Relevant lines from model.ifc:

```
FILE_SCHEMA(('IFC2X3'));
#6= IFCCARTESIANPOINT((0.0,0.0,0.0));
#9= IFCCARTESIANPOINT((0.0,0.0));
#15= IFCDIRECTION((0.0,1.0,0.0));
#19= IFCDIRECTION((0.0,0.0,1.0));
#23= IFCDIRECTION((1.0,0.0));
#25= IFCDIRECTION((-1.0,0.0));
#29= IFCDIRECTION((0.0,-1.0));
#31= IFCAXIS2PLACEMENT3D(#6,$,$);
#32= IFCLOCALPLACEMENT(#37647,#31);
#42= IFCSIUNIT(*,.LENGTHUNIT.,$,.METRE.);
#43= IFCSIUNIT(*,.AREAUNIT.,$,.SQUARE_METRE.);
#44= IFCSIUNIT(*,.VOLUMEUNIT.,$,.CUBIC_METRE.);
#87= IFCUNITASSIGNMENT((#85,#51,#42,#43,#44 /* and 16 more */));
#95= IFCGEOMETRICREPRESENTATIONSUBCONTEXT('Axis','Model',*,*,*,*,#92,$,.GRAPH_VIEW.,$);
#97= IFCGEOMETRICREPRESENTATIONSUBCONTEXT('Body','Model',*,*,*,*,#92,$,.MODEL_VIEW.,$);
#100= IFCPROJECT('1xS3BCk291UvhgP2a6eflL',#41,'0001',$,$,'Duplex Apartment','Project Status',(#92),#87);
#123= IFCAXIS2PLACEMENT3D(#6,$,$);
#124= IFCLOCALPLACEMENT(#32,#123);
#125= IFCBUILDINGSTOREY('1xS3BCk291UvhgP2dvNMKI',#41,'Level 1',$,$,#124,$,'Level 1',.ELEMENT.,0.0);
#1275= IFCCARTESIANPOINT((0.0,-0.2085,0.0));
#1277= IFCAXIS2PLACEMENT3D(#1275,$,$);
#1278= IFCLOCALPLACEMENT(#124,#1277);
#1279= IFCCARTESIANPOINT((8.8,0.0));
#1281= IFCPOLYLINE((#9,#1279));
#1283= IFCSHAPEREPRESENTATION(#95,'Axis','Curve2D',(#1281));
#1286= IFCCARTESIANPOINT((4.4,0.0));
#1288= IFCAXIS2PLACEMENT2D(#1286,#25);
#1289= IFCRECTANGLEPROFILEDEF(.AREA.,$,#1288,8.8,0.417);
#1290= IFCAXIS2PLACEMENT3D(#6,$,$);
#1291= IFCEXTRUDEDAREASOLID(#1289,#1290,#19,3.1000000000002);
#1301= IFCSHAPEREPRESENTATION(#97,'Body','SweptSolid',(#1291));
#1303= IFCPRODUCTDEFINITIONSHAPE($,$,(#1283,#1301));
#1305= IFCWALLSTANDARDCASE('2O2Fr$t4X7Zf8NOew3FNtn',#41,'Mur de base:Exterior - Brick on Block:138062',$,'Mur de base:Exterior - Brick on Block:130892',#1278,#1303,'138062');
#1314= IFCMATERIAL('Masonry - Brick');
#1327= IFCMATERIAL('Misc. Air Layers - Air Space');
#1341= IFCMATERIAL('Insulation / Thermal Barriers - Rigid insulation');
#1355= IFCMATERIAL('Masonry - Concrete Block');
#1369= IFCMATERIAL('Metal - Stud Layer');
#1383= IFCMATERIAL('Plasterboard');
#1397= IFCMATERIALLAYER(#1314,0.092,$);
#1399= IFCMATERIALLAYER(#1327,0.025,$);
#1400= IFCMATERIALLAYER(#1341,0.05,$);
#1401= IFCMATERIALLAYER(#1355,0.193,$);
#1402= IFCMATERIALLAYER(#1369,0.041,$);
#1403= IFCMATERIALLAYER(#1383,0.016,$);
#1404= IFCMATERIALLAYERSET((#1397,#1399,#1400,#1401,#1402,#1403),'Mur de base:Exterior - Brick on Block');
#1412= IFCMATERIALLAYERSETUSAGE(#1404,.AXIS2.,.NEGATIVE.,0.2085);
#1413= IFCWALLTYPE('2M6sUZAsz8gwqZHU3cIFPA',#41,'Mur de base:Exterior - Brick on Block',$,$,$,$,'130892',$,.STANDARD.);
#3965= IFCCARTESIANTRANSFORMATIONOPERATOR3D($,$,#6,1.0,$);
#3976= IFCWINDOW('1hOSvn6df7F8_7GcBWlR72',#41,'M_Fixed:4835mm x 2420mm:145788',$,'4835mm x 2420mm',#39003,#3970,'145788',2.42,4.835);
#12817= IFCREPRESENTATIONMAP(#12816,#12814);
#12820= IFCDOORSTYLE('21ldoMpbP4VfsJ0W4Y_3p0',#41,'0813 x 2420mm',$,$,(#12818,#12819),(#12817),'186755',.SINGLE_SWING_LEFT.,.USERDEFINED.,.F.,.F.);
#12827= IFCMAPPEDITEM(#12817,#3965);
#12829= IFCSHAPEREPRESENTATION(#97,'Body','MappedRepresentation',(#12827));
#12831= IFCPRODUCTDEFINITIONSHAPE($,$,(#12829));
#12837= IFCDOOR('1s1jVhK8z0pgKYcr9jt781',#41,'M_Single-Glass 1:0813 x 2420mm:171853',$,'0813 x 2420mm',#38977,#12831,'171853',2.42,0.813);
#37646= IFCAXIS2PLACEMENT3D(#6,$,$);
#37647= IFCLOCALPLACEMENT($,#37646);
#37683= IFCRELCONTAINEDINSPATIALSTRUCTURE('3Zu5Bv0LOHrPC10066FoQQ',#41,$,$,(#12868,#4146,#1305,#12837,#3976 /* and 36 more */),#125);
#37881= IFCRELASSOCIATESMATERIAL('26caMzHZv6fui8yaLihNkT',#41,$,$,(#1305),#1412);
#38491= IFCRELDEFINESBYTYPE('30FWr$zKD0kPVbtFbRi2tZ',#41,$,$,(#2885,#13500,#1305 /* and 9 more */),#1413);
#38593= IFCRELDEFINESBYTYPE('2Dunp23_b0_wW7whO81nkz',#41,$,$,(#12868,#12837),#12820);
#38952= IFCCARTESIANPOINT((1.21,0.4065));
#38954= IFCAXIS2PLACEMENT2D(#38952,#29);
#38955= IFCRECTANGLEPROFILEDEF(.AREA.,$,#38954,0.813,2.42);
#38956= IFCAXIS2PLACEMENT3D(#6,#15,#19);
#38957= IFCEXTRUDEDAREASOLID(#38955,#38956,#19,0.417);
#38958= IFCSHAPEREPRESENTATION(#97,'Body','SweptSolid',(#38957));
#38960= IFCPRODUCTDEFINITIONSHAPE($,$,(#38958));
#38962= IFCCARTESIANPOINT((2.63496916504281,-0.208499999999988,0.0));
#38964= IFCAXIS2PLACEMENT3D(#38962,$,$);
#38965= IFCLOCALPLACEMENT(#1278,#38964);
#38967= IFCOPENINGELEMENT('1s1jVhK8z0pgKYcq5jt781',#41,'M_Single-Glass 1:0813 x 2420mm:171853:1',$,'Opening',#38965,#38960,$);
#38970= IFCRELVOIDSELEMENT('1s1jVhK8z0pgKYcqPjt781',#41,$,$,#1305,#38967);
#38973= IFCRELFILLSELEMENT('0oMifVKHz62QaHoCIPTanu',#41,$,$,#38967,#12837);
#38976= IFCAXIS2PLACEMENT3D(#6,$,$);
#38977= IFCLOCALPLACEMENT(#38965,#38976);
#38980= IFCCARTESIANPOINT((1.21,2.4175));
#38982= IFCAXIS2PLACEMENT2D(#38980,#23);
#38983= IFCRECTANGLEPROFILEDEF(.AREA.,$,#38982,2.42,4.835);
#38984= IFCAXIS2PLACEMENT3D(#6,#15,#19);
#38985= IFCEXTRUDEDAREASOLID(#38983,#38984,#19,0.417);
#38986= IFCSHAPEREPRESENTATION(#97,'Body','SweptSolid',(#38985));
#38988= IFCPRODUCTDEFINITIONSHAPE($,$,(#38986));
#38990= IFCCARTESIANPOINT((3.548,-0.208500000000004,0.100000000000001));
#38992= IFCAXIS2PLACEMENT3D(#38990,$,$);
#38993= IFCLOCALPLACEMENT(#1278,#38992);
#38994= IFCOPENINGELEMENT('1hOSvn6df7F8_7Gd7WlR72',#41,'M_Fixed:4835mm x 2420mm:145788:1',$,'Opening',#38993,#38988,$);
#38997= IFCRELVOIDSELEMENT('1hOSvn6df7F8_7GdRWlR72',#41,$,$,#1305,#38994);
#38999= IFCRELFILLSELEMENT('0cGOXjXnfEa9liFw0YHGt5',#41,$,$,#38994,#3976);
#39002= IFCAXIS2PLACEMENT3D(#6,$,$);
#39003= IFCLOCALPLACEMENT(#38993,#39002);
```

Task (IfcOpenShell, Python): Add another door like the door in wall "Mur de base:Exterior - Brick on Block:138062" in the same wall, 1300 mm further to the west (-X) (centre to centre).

```python
import ifcopenshell
import ifcopenshell.api.feature
import ifcopenshell.api.geometry
import ifcopenshell.api.root
import ifcopenshell.geom
import ifcopenshell.util.element
import ifcopenshell.util.placement
import ifcopenshell.util.shape
import ifcopenshell.util.unit

model = ifcopenshell.open("model.ifc")
unit_scale = ifcopenshell.util.unit.calculate_unit_scale(model)
settings = ifcopenshell.geom.settings()


def volume(element):
    """Net volume in cubic metres, openings subtracted."""
    shape = ifcopenshell.geom.create_shape(settings, element)
    return ifcopenshell.util.shape.get_volume(shape.geometry)


def reuse_history(source, copy):
    """copy_class also copies each property set's owner history, people and application; keep the originals."""
    for rel in copy.IsDefinedBy:
        if rel.is_a("IfcRelDefinesByProperties") and (history := rel.RelatingPropertyDefinition.OwnerHistory):
            rel.RelatingPropertyDefinition.OwnerHistory = source.OwnerHistory
            ifcopenshell.util.element.remove_deep2(model, history)


door = model.by_guid("1s1jVhK8z0pgKYcr9jt781")
opening = door.FillsVoids[0].RelatingOpeningElement
wall = opening.VoidsElements[0].RelatingBuildingElement
before = volume(wall)
shift = ifcopenshell.util.placement.get_local_placement(wall.ObjectPlacement)[:3, 0] * -1.3 / unit_scale

# copy_class copies the void relationship, type, container and properties, but no geometry.
new_opening = ifcopenshell.api.root.copy_class(model, product=opening)
new_opening.Representation = ifcopenshell.util.element.copy_deep(
    model, opening.Representation, exclude=["IfcGeometricRepresentationContext", "IfcRepresentationMap"]
)
new_opening.Name = "M_Single-Glass 1:0813 x 2420mm"
new_door = ifcopenshell.api.root.copy_class(model, product=door)
new_door.Representation = ifcopenshell.util.element.copy_deep(
    model, door.Representation, exclude=["IfcGeometricRepresentationContext", "IfcRepresentationMap"]
)
new_door.Name = "M_Single-Glass 1:0813 x 2420mm"
new_door.Tag = None
reuse_history(door, new_door)
fills = ifcopenshell.api.feature.add_filling(model, opening=new_opening, element=new_door)
fills.OwnerHistory = new_door.OwnerHistory  # required in IFC2X3

for old, new in ((opening, new_opening), (door, new_door)):
    matrix = ifcopenshell.util.placement.get_local_placement(old.ObjectPlacement)
    matrix[:3, 3] += shift
    ifcopenshell.api.geometry.edit_object_placement(model, product=new, matrix=matrix, is_si=False)

after = volume(wall)

print(f"wall volume {before:.3f} -> {after:.3f} m3")

model.write("model_updated.ifc")
```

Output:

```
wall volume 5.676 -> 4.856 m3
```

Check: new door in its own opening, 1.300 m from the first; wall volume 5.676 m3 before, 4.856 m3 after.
